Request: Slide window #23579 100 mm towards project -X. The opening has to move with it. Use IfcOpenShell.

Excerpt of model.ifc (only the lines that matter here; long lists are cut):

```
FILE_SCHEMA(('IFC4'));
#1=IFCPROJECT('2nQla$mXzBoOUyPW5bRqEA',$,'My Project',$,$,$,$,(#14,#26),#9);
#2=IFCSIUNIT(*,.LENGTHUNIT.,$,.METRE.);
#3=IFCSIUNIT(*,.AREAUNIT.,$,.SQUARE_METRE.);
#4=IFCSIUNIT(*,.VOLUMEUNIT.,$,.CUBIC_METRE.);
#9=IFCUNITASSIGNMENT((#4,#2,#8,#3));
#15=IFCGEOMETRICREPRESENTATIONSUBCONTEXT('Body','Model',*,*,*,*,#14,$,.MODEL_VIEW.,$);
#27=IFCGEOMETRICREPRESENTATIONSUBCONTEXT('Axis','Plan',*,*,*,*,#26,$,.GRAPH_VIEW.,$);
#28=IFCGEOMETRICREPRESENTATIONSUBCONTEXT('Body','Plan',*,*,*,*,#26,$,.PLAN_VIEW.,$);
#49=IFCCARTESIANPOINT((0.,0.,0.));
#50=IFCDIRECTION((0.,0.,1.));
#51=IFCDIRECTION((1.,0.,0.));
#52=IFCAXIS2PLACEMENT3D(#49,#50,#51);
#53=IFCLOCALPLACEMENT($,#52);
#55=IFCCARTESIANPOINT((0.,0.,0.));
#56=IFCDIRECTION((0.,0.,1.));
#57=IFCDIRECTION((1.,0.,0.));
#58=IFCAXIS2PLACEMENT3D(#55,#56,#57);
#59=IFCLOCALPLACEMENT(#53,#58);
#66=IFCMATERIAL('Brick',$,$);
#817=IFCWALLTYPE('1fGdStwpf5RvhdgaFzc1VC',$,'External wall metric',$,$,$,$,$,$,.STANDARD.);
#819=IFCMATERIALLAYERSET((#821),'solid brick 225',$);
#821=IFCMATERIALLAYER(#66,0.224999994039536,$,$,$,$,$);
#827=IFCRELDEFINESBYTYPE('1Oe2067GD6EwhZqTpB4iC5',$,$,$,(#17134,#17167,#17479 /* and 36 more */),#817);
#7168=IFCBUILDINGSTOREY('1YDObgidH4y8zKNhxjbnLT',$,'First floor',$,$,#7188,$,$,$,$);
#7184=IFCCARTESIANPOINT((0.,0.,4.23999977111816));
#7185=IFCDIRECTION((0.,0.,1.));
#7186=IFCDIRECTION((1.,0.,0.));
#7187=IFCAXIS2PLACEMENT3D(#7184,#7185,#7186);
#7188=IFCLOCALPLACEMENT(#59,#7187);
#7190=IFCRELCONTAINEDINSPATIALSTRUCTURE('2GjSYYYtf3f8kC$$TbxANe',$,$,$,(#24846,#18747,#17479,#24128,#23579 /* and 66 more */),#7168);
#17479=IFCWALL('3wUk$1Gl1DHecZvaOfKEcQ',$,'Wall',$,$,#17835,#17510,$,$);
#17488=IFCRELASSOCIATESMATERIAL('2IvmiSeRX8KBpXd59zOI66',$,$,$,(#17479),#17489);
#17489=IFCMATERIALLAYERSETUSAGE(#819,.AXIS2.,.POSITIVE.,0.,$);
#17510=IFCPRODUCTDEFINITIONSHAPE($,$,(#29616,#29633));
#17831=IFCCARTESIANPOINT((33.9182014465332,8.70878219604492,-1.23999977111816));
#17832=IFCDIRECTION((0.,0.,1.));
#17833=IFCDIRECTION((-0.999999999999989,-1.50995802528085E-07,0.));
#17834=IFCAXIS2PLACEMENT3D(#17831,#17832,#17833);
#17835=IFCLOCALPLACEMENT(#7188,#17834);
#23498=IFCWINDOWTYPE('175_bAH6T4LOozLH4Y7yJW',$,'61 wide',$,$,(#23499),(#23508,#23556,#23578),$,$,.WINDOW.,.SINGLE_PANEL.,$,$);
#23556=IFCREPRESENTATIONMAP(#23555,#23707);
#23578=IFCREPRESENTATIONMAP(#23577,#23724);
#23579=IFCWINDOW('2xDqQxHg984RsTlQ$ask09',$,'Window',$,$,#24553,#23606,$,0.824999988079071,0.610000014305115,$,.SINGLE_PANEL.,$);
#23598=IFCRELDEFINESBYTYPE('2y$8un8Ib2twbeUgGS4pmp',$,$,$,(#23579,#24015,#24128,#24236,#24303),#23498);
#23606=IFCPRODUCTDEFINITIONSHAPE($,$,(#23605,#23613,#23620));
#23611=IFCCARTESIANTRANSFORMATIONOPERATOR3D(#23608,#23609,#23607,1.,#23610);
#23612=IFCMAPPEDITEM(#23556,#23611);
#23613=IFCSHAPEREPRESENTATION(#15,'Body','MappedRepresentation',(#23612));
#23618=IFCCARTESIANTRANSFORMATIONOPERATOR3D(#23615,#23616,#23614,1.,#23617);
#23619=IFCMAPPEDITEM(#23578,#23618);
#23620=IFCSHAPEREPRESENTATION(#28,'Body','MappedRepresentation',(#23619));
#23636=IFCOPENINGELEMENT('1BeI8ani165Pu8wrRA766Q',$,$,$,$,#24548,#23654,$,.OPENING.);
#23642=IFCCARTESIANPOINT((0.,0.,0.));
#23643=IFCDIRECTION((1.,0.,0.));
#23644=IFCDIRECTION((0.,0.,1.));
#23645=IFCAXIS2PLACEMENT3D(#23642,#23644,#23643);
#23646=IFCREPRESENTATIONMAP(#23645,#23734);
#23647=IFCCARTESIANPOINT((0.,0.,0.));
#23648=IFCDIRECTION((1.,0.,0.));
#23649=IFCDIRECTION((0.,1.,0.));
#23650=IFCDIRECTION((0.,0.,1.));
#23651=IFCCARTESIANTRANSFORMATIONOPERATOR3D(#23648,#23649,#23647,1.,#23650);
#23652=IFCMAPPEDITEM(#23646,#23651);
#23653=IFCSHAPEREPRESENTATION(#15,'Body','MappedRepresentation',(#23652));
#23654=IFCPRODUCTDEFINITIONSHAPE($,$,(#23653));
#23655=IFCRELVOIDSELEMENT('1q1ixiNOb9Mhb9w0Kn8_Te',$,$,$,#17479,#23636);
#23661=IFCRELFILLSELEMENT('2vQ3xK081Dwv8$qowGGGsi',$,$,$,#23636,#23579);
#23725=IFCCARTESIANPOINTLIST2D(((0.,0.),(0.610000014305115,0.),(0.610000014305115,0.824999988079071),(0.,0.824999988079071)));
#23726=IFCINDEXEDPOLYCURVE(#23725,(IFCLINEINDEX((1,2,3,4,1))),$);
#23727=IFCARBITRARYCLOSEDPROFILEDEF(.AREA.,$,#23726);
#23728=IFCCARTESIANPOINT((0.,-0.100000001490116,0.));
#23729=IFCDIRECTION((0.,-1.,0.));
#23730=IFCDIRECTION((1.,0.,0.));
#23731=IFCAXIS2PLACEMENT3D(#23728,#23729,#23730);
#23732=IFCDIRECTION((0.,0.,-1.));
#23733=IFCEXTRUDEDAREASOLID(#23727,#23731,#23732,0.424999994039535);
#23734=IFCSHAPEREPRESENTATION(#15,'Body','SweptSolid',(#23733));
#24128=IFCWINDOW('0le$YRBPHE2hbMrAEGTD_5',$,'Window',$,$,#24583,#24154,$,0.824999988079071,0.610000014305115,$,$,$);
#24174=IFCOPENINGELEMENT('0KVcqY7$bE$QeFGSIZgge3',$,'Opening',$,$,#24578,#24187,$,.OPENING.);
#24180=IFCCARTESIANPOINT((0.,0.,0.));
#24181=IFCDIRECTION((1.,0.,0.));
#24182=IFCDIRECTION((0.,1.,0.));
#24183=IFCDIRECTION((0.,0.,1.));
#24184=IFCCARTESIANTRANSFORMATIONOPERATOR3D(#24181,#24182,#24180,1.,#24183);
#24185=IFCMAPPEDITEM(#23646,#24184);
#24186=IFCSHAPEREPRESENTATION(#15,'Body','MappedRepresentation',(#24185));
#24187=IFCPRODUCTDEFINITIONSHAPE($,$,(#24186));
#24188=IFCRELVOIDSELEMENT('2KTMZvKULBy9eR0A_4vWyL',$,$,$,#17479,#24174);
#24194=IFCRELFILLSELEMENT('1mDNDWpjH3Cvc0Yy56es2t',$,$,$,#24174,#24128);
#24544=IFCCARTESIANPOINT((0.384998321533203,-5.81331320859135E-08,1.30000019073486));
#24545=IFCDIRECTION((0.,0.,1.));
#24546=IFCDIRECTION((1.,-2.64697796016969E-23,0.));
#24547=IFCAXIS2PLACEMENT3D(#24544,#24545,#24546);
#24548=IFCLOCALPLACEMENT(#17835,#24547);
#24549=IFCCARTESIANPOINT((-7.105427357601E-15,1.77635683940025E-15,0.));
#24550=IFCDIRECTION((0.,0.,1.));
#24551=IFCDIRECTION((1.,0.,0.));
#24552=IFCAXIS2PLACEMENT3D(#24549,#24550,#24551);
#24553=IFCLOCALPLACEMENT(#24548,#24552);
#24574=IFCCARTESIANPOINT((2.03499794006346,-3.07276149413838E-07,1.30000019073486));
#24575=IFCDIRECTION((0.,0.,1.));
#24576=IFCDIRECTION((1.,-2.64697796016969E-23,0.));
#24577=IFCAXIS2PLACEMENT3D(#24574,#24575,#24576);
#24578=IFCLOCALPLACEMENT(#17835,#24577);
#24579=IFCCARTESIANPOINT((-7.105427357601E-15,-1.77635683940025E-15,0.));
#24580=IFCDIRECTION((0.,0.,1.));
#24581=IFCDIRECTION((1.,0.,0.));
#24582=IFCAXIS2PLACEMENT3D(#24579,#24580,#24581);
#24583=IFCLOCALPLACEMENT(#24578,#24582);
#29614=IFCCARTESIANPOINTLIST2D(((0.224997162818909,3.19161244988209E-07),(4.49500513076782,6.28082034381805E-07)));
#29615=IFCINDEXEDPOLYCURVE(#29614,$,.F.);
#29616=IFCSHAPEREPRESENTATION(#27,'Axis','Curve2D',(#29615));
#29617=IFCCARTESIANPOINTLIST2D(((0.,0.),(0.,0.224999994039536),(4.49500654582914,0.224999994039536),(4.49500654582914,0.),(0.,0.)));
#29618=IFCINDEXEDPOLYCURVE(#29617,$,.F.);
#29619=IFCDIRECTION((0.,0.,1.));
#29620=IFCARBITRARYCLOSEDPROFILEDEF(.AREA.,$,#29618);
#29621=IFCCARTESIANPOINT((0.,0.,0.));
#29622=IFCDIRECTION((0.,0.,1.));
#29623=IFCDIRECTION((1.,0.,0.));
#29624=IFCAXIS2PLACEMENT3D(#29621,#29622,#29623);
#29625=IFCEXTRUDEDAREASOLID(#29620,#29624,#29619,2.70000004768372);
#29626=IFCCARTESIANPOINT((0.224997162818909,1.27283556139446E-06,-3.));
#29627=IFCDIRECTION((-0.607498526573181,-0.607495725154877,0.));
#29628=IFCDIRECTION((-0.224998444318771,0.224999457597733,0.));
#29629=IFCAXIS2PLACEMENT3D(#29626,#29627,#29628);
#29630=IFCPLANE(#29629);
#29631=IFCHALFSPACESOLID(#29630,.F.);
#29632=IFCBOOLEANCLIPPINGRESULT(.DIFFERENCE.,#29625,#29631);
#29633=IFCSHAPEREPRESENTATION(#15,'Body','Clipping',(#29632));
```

```python
import ifcopenshell
import ifcopenshell.api.geometry
import ifcopenshell.util.placement
import ifcopenshell.util.unit

model = ifcopenshell.open("model.ifc")
unit_scale = ifcopenshell.util.unit.calculate_unit_scale(model)

window = model.by_guid("2xDqQxHg984RsTlQ$ask09")
opening = window.FillsVoids[0].RelatingOpeningElement
wall = opening.VoidsElements[0].RelatingBuildingElement

wall_matrix = ifcopenshell.util.placement.get_local_placement(wall.ObjectPlacement)
shift = wall_matrix[:3, 0] * 0.1 / unit_scale
before = ifcopenshell.util.placement.get_local_placement(window.ObjectPlacement)[:3, 3].copy()

# The window is placed relative to its opening, so it follows when the opening moves.
matrix = ifcopenshell.util.placement.get_local_placement(opening.ObjectPlacement)
matrix[:3, 3] += shift
ifcopenshell.api.geometry.edit_object_placement(
    model, product=opening, matrix=matrix, is_si=False, should_transform_children=True
)

after = ifcopenshell.util.placement.get_local_placement(window.ObjectPlacement)[:3, 3]
print("window moved by", (after - before).round(3) + 0.0)

model.write("model-out.ifc")
```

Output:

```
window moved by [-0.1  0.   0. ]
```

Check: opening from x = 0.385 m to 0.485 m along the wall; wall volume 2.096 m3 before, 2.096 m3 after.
